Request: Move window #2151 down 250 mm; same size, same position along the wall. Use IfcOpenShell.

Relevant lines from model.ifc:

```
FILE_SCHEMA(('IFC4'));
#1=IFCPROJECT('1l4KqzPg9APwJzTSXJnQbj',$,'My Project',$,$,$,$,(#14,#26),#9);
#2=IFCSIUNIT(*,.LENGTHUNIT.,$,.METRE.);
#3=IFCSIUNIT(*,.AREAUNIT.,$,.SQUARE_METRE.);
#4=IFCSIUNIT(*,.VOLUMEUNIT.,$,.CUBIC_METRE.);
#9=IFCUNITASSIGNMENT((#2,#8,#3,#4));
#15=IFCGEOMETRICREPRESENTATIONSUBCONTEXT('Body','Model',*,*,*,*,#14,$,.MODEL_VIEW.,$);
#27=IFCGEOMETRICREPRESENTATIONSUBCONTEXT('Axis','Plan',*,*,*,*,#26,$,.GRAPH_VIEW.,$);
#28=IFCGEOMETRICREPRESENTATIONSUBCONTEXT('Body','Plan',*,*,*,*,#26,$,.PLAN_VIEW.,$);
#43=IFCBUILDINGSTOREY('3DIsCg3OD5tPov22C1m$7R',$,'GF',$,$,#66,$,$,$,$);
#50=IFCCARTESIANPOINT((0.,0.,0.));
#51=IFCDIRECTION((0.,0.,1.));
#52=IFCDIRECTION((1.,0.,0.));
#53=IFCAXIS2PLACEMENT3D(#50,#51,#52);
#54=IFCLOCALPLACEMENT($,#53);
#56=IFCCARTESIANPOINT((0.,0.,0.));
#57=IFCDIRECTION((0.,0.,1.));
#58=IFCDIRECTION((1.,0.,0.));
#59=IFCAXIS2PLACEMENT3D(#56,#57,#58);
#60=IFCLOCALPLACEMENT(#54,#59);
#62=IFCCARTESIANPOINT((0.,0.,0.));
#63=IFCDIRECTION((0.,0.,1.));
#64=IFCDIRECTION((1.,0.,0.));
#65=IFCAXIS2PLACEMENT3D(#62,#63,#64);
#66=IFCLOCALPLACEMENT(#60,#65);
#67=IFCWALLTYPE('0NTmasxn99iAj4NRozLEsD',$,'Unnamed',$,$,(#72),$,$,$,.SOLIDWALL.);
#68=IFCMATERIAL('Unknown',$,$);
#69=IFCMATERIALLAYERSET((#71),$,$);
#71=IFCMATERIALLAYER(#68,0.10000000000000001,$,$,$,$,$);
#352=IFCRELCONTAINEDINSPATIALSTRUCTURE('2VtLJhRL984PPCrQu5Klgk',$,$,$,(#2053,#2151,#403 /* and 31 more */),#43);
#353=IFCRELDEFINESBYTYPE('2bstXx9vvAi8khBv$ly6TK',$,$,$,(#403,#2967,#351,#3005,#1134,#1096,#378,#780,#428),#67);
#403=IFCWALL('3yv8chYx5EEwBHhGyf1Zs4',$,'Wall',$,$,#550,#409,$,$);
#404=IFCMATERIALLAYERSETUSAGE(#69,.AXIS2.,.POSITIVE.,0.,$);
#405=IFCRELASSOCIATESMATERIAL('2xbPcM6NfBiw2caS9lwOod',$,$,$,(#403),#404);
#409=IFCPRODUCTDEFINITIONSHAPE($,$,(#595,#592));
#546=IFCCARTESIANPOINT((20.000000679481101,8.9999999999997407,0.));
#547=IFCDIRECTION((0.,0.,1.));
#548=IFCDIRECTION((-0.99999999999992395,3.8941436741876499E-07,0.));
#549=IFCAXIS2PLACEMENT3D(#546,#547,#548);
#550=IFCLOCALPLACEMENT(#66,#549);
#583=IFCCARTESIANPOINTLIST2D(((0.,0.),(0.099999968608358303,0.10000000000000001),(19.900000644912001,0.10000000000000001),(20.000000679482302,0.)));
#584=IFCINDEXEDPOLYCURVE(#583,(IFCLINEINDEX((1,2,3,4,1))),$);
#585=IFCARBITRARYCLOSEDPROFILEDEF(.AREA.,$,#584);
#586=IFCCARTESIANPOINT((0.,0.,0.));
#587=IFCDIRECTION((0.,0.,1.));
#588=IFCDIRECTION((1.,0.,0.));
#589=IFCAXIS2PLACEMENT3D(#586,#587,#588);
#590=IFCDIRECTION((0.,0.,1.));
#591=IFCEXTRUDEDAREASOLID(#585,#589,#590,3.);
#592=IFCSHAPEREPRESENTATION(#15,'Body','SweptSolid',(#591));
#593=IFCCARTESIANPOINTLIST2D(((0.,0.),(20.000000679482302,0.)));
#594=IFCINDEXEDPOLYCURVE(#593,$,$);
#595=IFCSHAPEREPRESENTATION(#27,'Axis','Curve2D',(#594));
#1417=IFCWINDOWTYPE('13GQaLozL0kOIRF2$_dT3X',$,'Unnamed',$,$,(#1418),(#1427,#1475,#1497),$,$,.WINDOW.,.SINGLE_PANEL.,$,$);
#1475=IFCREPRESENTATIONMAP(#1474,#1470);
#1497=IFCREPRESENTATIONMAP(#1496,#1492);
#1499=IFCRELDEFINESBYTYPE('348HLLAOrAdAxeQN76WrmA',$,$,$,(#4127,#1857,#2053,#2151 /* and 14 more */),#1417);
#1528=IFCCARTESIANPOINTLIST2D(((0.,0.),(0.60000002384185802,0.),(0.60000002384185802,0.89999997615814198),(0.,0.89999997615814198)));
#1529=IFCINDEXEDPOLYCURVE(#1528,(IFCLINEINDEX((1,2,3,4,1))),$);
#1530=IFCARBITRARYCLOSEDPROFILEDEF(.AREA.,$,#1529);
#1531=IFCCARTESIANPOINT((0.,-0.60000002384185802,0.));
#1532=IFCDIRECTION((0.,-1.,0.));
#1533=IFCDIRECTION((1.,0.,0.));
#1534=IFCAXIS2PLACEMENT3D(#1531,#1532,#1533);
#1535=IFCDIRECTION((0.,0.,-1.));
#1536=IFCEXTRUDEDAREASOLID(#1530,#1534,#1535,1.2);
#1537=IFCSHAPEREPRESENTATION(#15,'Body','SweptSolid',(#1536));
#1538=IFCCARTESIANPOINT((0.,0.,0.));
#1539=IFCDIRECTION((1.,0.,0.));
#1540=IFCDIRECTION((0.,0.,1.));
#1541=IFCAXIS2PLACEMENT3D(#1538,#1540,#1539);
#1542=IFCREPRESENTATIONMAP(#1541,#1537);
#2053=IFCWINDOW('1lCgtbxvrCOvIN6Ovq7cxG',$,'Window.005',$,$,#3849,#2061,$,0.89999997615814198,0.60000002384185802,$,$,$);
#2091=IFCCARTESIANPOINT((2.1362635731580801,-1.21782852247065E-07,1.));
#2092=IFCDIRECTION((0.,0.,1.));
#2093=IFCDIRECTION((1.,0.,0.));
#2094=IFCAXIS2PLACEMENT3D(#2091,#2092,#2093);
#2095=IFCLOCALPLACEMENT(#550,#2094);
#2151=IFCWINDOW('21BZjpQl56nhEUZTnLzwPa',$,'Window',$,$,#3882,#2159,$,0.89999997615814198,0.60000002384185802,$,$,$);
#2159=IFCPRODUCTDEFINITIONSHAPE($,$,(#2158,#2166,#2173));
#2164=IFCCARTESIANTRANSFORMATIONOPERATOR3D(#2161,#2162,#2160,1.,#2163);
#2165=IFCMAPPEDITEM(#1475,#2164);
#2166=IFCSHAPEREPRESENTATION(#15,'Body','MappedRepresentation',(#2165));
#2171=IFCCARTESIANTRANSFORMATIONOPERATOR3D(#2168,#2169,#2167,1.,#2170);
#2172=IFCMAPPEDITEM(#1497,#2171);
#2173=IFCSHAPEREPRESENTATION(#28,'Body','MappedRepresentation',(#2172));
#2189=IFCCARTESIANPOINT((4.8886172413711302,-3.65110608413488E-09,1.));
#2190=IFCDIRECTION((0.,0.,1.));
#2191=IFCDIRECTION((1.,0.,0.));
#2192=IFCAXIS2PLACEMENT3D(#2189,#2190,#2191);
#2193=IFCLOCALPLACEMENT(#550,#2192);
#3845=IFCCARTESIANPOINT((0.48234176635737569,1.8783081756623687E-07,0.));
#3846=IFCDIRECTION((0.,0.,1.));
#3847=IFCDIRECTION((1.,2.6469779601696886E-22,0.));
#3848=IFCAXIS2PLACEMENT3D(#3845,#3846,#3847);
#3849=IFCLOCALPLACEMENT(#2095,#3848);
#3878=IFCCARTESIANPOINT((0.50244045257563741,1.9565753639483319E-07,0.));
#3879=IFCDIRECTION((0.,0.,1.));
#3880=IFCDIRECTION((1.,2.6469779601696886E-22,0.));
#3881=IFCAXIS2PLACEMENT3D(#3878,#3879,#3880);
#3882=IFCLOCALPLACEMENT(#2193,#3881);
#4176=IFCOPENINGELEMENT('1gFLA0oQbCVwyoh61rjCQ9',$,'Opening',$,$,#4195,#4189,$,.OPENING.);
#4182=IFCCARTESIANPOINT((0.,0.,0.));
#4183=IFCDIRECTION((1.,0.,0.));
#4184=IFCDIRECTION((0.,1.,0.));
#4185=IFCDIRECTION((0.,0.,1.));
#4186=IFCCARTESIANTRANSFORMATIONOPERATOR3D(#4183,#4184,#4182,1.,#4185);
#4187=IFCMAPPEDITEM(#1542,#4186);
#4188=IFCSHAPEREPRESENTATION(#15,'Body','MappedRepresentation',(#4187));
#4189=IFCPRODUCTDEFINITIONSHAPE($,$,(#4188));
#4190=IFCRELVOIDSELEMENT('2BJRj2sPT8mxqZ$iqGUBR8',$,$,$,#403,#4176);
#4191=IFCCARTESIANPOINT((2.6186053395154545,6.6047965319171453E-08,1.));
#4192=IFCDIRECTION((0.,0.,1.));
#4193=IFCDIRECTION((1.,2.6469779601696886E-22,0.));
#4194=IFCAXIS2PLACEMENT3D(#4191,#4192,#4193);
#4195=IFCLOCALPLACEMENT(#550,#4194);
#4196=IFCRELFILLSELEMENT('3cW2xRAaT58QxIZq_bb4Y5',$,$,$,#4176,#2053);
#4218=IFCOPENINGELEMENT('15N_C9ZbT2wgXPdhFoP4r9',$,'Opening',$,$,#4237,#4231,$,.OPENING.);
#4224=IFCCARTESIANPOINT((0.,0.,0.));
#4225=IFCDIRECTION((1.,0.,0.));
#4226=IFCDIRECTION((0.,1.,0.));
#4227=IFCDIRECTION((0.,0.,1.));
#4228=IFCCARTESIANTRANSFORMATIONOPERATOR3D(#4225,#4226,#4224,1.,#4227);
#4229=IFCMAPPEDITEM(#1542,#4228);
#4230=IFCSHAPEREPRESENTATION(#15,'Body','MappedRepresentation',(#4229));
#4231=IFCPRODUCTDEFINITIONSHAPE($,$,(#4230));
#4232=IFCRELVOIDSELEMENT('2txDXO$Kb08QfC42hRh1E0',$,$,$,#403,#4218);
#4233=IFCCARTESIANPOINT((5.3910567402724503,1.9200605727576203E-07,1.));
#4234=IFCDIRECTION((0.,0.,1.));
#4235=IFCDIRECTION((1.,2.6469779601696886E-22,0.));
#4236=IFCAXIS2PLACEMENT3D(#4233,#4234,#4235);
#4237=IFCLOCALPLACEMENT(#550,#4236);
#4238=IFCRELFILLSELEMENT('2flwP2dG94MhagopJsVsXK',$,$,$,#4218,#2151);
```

```python
import numpy as np
import ifcopenshell
import ifcopenshell.api.geometry
import ifcopenshell.util.placement
import ifcopenshell.util.unit

model = ifcopenshell.open("model.ifc")
unit_scale = ifcopenshell.util.unit.calculate_unit_scale(model)

window = model.by_id(2151)
opening = window.FillsVoids[0].RelatingOpeningElement
dz = -0.25

shift = np.array([0.0, 0.0, dz])
# The window is not placed relative to its opening, so move both.
for product in (opening, window):
    matrix = ifcopenshell.util.placement.get_local_placement(product.ObjectPlacement)
    matrix[:3, 3] += shift
    ifcopenshell.api.geometry.edit_object_placement(model, product=product, matrix=matrix, is_si=False)

print(f"moved by {dz * unit_scale:+.3f} m")

model.write("model_edited.ifc")
```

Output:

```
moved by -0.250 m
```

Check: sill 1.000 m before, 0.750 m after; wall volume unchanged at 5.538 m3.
